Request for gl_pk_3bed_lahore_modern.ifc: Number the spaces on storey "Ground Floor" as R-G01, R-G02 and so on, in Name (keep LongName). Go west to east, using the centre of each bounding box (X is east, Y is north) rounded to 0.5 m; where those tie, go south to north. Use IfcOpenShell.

First a look at what the model holds.

```python
import ifcopenshell
import ifcopenshell.util.element
import ifcopenshell.util.placement

model = ifcopenshell.open("gl_pk_3bed_lahore_modern.ifc")
print(model.schema)
storey = next(s for s in model.by_type("IfcBuildingStorey") if s.Name == "Ground Floor")
spaces = [e for e in ifcopenshell.util.element.get_decomposition(storey) if e.is_a("IfcSpace")]
for e in sorted(spaces, key=lambda e: e.id()):
    origin = ifcopenshell.util.placement.get_local_placement(e.ObjectPlacement)[:3, 3]
    print(e.id(), e.Name, e.LongName, origin.round(2) + 0.0, sep=" | ")
```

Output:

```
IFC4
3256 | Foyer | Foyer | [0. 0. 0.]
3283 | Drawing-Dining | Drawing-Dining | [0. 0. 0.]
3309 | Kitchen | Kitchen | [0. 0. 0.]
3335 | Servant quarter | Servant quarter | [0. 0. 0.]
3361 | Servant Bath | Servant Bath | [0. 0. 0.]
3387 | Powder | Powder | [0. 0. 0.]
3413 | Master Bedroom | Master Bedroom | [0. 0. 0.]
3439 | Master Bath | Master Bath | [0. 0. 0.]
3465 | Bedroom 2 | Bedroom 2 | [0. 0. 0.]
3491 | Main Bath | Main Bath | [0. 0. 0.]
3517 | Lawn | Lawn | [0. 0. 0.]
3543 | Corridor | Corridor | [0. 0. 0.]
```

```python
import ifcopenshell
import ifcopenshell.geom
import ifcopenshell.util.element
import ifcopenshell.util.shape

model = ifcopenshell.open("gl_pk_3bed_lahore_modern.ifc")
settings = ifcopenshell.geom.settings()
settings.set("use-world-coords", True)


def centre(element):
    shape = ifcopenshell.geom.create_shape(settings, element)
    return ifcopenshell.util.shape.get_bbox_centroid(shape.geometry)


storey = next(s for s in model.by_type("IfcBuildingStorey") if s.Name == "Ground Floor")
spaces = [e for e in ifcopenshell.util.element.get_decomposition(storey) if e.is_a("IfcSpace")]

# Insertion points can sit at a corner or the storey origin, so sort by the geometry (in metres).
centres = {e: centre(e) for e in spaces}
spaces.sort(key=lambda e: (round(centres[e][0] / 0.5), centres[e][1]))

for i, e in enumerate(spaces, start=1):
    number = f"R-G{i:02d}"
    e.Name = number
    print(e.id(), number)

model.write("gl_pk_3bed_lahore_modern_v2.ifc")
```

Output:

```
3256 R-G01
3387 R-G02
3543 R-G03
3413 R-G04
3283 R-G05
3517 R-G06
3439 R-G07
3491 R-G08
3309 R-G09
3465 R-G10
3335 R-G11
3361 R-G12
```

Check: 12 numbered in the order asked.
